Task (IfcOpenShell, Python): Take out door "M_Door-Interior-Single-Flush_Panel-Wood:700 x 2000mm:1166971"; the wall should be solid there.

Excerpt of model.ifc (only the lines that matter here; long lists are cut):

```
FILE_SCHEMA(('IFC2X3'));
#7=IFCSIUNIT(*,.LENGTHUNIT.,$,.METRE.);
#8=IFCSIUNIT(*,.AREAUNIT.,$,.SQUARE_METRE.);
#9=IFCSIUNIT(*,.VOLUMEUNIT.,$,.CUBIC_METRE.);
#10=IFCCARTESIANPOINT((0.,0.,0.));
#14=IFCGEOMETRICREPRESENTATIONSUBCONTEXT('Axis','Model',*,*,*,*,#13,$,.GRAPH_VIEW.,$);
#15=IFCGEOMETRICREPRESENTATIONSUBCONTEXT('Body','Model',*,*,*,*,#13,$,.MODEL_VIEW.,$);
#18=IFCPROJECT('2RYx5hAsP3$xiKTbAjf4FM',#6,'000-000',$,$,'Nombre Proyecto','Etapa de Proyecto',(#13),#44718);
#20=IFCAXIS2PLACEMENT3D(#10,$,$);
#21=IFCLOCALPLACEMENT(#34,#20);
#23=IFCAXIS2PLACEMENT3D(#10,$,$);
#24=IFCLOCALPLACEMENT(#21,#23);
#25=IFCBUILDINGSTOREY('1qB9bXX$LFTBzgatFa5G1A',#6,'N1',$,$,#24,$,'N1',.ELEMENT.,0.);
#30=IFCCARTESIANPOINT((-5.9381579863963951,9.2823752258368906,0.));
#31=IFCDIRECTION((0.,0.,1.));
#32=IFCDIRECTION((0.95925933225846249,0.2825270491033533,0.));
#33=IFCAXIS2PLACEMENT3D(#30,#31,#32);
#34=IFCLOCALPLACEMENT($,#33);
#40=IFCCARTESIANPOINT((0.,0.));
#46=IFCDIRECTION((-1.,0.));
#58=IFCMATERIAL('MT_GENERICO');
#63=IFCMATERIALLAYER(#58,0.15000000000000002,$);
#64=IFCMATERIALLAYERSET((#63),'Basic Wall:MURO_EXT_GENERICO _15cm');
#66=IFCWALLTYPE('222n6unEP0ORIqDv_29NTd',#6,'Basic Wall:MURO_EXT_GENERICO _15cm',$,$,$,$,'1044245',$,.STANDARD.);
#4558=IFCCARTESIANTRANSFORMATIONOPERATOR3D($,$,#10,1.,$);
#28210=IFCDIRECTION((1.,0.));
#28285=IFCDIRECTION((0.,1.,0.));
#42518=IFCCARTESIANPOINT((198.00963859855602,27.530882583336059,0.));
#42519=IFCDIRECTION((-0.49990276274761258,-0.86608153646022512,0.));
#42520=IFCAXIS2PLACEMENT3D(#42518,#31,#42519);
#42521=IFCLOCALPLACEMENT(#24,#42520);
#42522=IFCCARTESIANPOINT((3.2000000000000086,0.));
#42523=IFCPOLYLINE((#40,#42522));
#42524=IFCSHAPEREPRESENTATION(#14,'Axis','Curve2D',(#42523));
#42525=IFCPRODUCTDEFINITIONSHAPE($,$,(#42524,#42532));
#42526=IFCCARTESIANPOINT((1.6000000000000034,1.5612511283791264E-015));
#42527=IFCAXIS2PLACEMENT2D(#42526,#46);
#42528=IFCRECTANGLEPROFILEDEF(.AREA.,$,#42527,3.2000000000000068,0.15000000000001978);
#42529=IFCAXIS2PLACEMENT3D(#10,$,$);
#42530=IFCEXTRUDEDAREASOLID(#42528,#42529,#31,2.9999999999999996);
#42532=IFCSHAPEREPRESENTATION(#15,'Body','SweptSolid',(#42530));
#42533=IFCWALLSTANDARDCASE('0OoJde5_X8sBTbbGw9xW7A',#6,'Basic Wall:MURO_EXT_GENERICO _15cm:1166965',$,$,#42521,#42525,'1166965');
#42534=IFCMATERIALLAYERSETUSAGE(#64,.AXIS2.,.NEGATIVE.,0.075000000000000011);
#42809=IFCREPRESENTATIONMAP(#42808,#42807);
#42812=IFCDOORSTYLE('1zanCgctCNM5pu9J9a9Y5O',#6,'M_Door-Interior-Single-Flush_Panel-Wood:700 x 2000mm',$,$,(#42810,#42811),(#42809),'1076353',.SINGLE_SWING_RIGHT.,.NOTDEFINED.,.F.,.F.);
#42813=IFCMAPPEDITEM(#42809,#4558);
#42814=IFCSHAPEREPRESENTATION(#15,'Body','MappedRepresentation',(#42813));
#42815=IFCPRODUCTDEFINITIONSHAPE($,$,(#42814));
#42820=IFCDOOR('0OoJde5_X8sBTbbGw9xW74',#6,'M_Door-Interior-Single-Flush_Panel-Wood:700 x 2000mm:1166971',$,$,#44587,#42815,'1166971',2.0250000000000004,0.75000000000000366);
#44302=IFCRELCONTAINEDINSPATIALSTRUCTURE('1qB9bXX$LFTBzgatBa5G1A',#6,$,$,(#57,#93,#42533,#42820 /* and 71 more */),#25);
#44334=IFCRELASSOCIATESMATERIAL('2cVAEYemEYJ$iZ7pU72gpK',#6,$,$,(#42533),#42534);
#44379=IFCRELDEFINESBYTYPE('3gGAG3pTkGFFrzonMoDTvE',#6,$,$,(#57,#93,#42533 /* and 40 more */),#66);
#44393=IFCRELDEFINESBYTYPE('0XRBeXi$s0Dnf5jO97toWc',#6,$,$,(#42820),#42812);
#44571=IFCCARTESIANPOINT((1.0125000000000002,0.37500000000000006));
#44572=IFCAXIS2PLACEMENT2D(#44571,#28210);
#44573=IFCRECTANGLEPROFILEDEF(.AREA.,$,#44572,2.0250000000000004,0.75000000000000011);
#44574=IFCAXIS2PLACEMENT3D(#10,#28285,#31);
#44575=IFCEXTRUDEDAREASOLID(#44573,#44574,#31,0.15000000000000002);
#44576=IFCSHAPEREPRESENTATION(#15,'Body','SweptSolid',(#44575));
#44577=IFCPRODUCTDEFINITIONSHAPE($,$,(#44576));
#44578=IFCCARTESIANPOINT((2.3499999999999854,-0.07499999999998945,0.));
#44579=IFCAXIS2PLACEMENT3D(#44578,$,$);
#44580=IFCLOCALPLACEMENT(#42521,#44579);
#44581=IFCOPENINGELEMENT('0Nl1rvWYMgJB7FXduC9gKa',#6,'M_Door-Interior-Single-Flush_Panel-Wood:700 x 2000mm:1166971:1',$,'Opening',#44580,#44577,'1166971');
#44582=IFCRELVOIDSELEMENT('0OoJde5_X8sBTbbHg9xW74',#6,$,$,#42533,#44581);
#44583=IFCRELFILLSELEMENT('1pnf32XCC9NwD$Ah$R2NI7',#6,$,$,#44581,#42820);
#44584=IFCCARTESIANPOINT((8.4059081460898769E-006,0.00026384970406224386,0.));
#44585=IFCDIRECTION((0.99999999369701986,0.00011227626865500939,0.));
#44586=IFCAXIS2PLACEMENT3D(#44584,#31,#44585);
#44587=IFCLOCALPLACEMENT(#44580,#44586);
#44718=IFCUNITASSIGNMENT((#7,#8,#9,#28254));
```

```python
import ifcopenshell
import ifcopenshell.api.feature
import ifcopenshell.api.root
import ifcopenshell.geom
import ifcopenshell.util.shape

model = ifcopenshell.open("model.ifc")
settings = ifcopenshell.geom.settings()


def volume(element):
    """Net volume in cubic metres, openings subtracted."""
    shape = ifcopenshell.geom.create_shape(settings, element)
    return ifcopenshell.util.shape.get_volume(shape.geometry)


door = model.by_guid("0OoJde5_X8sBTbbGw9xW74")
opening = door.FillsVoids[0].RelatingOpeningElement
wall = opening.VoidsElements[0].RelatingBuildingElement
before = volume(wall)

ifcopenshell.api.root.remove_product(model, product=door)
ifcopenshell.api.feature.remove_feature(model, feature=opening)

after = volume(wall)

print(f"wall volume {before:.3f} -> {after:.3f} m3")

model.write("model-out.ifc")
```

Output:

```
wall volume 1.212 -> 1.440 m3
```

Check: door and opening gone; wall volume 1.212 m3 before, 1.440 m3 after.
